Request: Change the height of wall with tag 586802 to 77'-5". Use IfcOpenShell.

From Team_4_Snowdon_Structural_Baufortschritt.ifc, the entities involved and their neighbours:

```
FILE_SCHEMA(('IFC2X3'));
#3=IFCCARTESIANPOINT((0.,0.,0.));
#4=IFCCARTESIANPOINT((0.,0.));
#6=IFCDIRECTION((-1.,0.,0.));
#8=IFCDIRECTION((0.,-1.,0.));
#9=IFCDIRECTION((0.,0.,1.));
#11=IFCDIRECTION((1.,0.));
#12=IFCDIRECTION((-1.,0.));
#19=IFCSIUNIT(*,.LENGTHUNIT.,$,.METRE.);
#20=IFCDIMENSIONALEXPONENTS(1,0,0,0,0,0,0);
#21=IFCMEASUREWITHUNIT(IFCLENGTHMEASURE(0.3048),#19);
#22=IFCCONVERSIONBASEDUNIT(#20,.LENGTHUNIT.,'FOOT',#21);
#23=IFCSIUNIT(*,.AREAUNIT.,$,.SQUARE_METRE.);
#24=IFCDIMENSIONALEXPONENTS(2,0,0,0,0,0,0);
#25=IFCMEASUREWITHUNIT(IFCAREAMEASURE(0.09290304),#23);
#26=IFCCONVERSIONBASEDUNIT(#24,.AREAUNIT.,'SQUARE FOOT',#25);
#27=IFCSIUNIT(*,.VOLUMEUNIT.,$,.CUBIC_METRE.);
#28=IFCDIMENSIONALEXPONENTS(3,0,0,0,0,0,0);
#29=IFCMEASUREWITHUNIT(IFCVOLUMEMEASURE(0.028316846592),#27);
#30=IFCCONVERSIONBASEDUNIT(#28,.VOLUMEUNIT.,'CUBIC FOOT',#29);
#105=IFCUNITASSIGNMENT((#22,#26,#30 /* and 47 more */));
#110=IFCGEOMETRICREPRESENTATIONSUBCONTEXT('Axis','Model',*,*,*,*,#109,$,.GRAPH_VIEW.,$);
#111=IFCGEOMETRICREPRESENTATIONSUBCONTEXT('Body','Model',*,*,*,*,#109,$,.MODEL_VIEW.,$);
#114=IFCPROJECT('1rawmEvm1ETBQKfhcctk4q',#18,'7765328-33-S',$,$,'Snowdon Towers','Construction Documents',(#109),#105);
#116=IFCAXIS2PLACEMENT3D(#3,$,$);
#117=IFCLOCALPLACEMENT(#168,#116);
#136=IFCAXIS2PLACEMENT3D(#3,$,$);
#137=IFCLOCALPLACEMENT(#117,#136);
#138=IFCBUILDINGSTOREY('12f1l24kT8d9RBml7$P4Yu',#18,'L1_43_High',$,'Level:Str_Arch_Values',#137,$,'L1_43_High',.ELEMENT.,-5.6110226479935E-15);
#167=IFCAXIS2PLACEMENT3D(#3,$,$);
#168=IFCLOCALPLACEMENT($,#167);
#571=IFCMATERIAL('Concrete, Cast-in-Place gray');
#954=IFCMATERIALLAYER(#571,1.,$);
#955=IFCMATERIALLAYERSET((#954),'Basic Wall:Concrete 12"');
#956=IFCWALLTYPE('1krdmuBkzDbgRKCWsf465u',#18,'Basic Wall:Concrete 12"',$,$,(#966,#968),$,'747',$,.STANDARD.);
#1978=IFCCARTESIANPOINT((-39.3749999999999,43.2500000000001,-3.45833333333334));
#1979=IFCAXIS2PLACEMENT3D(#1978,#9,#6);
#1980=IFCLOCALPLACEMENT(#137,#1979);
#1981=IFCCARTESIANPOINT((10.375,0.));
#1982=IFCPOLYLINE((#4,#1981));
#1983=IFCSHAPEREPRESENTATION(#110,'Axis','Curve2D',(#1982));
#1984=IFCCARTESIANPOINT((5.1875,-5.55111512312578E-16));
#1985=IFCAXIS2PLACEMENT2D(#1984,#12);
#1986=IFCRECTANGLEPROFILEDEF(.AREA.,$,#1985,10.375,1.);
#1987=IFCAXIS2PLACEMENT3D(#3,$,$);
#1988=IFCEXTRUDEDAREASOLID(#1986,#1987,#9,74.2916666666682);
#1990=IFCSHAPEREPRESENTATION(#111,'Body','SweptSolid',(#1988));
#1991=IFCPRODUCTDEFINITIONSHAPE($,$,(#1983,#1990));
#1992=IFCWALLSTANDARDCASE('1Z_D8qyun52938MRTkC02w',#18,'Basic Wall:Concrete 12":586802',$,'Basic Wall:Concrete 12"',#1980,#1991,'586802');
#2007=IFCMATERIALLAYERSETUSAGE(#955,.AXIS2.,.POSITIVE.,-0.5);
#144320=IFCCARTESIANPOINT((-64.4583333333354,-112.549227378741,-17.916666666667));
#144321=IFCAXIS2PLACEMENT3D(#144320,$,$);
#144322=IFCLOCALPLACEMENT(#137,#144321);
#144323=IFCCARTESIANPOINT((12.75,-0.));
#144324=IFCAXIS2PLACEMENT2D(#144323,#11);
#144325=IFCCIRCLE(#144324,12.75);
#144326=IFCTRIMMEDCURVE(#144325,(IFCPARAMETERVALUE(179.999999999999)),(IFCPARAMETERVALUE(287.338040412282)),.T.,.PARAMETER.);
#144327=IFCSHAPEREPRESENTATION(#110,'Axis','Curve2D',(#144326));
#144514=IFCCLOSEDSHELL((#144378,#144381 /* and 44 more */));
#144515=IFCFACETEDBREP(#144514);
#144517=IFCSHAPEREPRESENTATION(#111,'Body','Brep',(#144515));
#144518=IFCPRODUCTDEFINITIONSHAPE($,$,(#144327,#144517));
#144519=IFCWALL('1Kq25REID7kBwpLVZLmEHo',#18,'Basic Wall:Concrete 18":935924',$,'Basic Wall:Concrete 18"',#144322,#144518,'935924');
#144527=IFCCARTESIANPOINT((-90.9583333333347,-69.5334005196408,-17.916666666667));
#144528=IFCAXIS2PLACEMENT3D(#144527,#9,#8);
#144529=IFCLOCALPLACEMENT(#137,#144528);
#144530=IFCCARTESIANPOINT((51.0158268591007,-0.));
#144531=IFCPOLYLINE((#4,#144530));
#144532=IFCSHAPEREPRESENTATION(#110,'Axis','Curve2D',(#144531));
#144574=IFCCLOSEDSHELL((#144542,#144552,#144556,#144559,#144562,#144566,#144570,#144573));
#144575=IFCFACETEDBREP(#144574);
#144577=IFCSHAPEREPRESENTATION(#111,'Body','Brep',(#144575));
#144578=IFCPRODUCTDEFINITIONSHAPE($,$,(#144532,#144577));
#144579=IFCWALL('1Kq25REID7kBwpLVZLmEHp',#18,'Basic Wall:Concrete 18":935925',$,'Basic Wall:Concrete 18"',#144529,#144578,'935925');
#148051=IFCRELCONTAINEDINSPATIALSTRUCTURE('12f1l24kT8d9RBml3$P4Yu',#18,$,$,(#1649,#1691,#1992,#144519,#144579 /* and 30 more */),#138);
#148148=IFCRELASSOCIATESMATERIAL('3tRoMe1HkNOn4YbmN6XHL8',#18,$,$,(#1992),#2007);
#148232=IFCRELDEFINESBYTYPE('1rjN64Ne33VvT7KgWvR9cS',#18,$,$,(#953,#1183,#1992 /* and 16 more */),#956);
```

```python
import ifcopenshell
import ifcopenshell.geom
import ifcopenshell.util.representation
import ifcopenshell.util.shape
import ifcopenshell.util.unit

model = ifcopenshell.open("Team_4_Snowdon_Structural_Baufortschritt.ifc")
unit_scale = ifcopenshell.util.unit.calculate_unit_scale(model)
settings = ifcopenshell.geom.settings()


def volume(element):
    """Net volume in cubic metres, openings subtracted."""
    shape = ifcopenshell.geom.create_shape(settings, element)
    return ifcopenshell.util.shape.get_volume(shape.geometry)


wall = model.by_guid("1Z_D8qyun52938MRTkC02w")
before = volume(wall)

body = ifcopenshell.util.representation.get_representation(wall, "Model", "Body")
solid = body.Items[0]
old_height = solid.Depth
solid.Depth = 929 * 0.0254 / unit_scale
after = volume(wall)

print(f"height {old_height:g} -> {solid.Depth:g}, volume {before:.3f} -> {after:.3f} m3")

model.write("Team_4_Snowdon_Structural_Baufortschritt-out.ifc")
```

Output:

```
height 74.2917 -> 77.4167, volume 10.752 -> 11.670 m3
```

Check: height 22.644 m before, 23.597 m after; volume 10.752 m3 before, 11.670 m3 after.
